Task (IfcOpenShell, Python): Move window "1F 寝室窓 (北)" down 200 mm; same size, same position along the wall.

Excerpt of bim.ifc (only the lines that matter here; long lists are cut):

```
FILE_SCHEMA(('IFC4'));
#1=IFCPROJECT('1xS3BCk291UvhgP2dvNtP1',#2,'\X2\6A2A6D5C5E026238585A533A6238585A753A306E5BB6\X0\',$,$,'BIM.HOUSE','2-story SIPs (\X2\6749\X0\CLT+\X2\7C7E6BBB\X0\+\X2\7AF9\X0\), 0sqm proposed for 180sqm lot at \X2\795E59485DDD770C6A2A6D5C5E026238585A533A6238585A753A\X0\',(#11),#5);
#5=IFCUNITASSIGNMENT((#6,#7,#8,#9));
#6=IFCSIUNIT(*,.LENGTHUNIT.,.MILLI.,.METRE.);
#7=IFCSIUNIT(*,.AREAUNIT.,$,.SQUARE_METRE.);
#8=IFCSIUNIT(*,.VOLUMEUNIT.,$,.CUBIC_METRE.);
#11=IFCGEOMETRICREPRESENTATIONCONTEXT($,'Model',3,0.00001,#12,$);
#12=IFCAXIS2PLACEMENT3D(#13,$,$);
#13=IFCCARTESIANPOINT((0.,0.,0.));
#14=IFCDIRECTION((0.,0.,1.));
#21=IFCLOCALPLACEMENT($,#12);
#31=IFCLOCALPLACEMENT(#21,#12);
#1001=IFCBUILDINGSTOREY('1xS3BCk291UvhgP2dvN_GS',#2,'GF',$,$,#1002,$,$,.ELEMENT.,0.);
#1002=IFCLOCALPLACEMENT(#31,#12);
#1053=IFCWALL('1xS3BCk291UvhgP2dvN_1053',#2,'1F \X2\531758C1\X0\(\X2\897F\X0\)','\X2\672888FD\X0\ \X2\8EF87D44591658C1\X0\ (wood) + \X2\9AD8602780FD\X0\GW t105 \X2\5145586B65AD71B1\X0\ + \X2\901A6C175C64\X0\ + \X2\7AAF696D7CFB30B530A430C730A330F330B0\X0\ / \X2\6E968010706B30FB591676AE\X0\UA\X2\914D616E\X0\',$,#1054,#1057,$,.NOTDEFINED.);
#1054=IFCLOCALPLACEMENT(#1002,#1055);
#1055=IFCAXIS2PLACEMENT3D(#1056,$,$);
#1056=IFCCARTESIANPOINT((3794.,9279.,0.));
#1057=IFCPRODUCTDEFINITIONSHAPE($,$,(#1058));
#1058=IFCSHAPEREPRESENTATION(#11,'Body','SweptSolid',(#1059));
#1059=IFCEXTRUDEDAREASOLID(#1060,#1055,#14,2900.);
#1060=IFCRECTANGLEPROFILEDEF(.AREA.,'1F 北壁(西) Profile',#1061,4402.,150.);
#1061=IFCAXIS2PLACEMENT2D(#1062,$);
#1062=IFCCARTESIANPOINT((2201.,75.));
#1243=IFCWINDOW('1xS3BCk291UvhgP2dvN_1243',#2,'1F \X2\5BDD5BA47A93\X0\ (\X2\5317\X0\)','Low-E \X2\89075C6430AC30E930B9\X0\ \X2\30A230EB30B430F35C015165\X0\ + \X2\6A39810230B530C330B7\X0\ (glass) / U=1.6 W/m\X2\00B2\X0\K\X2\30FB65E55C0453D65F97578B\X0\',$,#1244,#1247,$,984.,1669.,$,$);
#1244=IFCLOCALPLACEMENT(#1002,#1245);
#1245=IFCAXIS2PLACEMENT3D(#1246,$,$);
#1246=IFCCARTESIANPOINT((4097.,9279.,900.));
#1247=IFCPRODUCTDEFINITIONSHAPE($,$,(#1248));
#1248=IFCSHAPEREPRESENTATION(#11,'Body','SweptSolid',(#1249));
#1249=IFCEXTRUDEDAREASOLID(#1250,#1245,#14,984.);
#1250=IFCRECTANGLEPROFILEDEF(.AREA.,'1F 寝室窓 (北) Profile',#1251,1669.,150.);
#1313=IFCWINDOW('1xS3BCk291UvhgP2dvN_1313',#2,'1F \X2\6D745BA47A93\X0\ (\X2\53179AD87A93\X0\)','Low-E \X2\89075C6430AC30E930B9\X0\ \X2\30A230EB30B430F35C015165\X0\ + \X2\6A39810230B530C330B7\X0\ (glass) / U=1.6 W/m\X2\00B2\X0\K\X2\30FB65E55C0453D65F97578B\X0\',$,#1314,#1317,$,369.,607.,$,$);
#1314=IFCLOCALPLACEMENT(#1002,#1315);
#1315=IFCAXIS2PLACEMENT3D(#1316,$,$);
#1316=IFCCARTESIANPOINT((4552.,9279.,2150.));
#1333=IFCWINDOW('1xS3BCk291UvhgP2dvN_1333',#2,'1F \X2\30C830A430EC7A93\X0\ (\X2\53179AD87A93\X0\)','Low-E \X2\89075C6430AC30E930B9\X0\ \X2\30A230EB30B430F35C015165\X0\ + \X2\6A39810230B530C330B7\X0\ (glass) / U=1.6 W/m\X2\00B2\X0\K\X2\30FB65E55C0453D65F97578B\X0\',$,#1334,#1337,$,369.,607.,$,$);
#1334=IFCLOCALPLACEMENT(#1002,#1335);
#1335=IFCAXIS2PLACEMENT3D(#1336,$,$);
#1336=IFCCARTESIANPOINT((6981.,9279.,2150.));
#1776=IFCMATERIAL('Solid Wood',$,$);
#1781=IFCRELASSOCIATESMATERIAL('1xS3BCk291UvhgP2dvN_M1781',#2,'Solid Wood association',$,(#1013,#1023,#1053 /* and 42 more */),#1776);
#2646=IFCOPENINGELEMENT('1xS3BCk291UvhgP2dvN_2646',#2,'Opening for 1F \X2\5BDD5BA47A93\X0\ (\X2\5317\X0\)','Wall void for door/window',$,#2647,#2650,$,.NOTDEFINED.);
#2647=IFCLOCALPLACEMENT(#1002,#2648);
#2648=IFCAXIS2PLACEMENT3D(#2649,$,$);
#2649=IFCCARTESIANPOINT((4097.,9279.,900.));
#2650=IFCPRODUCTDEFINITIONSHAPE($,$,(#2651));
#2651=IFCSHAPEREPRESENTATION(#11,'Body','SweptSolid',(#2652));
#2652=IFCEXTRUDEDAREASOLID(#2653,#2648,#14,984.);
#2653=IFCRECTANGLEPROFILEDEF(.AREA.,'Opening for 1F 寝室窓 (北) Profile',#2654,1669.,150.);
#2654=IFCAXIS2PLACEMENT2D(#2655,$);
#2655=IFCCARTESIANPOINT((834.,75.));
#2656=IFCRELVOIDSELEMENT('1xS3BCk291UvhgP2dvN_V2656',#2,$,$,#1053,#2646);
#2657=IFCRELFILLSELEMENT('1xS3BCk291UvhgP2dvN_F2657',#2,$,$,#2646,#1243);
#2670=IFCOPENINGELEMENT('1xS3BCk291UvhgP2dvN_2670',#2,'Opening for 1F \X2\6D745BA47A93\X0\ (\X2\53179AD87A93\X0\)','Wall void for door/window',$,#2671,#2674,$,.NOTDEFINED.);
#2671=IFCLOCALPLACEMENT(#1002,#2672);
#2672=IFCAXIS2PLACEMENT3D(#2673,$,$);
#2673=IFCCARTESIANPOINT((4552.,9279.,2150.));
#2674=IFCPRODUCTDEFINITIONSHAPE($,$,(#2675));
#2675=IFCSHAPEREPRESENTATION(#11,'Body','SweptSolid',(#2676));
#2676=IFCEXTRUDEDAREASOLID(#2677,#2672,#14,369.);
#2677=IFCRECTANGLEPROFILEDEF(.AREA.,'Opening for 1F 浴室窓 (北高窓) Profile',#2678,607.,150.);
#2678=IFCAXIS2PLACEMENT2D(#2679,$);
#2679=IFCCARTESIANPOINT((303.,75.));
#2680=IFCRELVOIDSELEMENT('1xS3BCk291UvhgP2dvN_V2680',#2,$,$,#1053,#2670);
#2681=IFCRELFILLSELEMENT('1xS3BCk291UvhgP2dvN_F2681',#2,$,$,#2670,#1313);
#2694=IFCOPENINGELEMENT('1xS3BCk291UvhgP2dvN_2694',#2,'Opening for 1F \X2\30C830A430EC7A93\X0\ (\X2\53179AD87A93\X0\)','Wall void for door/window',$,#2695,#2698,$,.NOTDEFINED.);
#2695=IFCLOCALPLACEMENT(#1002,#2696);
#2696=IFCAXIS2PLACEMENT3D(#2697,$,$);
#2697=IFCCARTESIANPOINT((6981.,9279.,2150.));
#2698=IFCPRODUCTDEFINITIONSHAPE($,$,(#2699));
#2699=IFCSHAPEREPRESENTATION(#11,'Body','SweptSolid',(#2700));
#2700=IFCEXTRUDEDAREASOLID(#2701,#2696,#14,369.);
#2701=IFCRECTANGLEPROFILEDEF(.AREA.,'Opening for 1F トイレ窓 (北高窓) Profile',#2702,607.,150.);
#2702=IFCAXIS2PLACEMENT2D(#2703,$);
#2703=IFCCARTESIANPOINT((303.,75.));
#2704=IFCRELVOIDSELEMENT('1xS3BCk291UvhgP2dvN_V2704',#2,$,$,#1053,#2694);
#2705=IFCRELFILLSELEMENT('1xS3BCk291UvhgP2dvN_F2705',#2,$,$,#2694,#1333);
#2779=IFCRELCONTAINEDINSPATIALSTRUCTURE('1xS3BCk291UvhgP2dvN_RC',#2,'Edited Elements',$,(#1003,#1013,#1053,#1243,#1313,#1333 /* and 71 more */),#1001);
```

```python
import numpy as np
import ifcopenshell
import ifcopenshell.api.geometry
import ifcopenshell.util.placement
import ifcopenshell.util.unit

model = ifcopenshell.open("bim.ifc")
unit_scale = ifcopenshell.util.unit.calculate_unit_scale(model)

window = model.by_guid("1xS3BCk291UvhgP2dvN_1243")
opening = window.FillsVoids[0].RelatingOpeningElement
dz = -200.0

shift = np.array([0.0, 0.0, dz])
# The window is not placed relative to its opening, so move both.
for product in (opening, window):
    matrix = ifcopenshell.util.placement.get_local_placement(product.ObjectPlacement)
    matrix[:3, 3] += shift
    ifcopenshell.api.geometry.edit_object_placement(model, product=product, matrix=matrix, is_si=False)

print(f"moved by {dz * unit_scale:+.3f} m")

model.write("bim_edited.ifc")
```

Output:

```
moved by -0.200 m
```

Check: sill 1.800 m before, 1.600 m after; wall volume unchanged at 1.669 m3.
